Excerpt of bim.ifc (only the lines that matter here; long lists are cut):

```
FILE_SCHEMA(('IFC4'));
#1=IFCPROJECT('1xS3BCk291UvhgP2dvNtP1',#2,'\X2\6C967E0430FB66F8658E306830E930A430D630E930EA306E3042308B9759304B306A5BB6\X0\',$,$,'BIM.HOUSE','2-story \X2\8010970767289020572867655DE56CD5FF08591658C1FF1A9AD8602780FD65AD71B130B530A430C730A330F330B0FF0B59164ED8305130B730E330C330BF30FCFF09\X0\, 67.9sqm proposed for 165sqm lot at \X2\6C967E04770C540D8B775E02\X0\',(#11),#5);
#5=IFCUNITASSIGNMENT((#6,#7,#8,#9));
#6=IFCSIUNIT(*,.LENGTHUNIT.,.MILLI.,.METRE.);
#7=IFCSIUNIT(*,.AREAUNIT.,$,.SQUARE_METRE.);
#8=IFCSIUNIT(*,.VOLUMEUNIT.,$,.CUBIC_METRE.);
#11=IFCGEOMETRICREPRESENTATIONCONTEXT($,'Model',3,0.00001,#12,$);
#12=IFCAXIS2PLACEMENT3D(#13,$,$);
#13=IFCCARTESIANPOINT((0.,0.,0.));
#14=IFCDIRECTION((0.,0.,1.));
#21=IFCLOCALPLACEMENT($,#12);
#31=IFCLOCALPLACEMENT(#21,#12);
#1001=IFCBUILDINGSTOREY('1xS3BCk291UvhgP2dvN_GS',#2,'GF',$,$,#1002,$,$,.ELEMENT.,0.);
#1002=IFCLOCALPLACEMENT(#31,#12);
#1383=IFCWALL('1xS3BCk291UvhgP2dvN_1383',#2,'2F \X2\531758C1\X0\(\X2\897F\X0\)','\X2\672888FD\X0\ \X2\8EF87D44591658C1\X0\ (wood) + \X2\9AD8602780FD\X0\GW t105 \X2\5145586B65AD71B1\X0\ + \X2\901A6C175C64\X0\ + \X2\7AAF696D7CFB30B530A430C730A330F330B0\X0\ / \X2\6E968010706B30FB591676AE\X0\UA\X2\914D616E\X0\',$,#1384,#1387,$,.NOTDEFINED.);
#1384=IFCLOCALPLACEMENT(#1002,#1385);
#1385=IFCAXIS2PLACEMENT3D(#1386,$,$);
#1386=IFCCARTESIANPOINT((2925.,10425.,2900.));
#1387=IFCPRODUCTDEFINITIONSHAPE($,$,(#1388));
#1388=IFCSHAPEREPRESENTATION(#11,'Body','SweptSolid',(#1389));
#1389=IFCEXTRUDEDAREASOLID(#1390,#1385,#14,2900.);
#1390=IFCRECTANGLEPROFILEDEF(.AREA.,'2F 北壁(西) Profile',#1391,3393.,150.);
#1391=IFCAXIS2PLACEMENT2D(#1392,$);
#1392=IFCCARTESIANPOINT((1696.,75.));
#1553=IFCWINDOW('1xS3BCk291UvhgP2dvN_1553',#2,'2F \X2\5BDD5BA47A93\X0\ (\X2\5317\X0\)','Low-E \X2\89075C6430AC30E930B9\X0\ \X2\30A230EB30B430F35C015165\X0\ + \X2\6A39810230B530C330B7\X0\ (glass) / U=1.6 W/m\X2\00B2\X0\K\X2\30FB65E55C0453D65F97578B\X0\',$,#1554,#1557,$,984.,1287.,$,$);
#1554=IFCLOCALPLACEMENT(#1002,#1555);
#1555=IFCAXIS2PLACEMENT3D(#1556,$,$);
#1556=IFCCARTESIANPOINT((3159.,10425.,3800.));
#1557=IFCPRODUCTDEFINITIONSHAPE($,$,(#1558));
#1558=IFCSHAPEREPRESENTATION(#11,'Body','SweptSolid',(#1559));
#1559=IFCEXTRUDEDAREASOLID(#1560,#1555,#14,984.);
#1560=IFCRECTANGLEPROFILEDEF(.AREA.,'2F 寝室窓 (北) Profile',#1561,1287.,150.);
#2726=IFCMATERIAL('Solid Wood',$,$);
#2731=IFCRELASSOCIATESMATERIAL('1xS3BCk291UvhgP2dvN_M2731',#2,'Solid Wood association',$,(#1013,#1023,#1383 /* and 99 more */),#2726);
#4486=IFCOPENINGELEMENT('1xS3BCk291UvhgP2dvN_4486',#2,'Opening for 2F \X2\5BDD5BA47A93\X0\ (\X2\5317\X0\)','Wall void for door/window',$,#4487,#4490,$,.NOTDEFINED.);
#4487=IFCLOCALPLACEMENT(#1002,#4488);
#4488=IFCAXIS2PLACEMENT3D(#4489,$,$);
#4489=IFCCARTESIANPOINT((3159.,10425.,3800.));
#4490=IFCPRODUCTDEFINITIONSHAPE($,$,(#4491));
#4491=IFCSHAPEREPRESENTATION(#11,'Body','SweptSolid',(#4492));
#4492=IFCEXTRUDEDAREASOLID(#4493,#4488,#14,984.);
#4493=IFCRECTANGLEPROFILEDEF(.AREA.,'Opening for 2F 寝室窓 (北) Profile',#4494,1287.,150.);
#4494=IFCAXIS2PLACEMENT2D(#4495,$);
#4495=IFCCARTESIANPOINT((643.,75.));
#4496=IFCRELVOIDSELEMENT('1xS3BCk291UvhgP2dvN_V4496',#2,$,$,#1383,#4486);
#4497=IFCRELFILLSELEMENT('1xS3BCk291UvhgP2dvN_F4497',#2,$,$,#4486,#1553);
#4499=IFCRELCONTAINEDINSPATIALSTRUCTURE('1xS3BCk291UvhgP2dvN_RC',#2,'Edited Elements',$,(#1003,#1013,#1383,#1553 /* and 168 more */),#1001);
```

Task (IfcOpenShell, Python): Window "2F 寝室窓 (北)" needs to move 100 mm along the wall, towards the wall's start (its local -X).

```python
import ifcopenshell
import ifcopenshell.api.geometry
import ifcopenshell.util.placement
import ifcopenshell.util.unit

model = ifcopenshell.open("bim.ifc")
unit_scale = ifcopenshell.util.unit.calculate_unit_scale(model)

window = model.by_guid("1xS3BCk291UvhgP2dvN_1553")
opening = window.FillsVoids[0].RelatingOpeningElement
wall = opening.VoidsElements[0].RelatingBuildingElement

wall_matrix = ifcopenshell.util.placement.get_local_placement(wall.ObjectPlacement)
shift = wall_matrix[:3, 0] * -0.1 / unit_scale
before = ifcopenshell.util.placement.get_local_placement(window.ObjectPlacement)[:3, 3].copy()

# The window is not placed relative to its opening, so move both.
for product in (opening, window):
    matrix = ifcopenshell.util.placement.get_local_placement(product.ObjectPlacement)
    matrix[:3, 3] += shift
    ifcopenshell.api.geometry.edit_object_placement(model, product=product, matrix=matrix, is_si=False)

after = ifcopenshell.util.placement.get_local_placement(window.ObjectPlacement)[:3, 3]
print("window moved by", (after - before).round(3) + 0.0)

model.write("bim_rev.ifc")
```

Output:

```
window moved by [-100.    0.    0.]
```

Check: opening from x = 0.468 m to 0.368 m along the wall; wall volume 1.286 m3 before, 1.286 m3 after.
